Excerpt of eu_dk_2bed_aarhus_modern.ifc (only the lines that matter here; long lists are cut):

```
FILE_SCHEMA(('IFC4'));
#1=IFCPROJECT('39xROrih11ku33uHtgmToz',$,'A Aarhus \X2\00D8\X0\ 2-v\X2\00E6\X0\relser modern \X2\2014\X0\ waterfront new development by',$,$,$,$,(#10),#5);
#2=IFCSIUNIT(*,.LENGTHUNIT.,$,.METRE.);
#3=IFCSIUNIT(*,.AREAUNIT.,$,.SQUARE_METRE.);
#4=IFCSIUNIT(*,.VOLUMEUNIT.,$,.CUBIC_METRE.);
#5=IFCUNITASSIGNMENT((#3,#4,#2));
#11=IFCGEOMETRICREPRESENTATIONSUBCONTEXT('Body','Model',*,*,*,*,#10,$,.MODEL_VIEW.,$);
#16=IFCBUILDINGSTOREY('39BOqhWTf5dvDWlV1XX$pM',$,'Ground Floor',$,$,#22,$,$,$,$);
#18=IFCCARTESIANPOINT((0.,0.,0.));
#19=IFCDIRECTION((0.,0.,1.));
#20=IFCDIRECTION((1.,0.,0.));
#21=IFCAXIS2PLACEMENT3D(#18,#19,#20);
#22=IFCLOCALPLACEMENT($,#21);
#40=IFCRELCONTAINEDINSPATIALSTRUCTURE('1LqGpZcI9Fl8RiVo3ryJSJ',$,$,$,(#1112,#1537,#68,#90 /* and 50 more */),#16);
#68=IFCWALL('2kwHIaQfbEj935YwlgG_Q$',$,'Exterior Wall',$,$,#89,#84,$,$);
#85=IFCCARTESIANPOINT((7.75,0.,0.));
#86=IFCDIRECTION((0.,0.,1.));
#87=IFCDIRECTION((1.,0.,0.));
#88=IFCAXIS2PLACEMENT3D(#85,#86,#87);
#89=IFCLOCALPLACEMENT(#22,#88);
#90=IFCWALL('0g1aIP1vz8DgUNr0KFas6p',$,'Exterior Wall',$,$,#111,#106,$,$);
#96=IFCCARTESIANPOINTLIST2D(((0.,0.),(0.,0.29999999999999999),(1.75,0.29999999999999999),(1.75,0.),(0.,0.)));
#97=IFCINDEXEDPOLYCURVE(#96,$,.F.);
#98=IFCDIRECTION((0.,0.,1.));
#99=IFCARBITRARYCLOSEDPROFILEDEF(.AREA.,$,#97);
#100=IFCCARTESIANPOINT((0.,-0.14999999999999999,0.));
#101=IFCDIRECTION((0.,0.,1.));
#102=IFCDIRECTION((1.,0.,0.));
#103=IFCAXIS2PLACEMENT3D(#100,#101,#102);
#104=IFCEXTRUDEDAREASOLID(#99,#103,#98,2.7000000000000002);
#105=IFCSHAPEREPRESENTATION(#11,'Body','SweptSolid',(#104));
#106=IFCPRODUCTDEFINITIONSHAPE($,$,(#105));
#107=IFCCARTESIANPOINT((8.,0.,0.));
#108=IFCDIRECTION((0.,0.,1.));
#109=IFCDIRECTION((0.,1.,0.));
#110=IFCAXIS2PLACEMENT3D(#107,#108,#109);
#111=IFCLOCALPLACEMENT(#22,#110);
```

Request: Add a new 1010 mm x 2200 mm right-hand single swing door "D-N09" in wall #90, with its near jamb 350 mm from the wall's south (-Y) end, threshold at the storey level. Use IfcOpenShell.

```python
import numpy as np
import ifcopenshell
import ifcopenshell.api.feature
import ifcopenshell.api.geometry
import ifcopenshell.api.root
import ifcopenshell.api.spatial
import ifcopenshell.geom
import ifcopenshell.util.element
import ifcopenshell.util.placement
import ifcopenshell.util.representation
import ifcopenshell.util.shape
import ifcopenshell.util.unit

model = ifcopenshell.open("eu_dk_2bed_aarhus_modern.ifc")
unit_scale = ifcopenshell.util.unit.calculate_unit_scale(model)
settings = ifcopenshell.geom.settings()


def volume(element):
    """Net volume in cubic metres, openings subtracted."""
    shape = ifcopenshell.geom.create_shape(settings, element)
    return ifcopenshell.util.shape.get_volume(shape.geometry)


wall = model.by_guid("0g1aIP1vz8DgUNr0KFas6p")
storey = ifcopenshell.util.element.get_container(wall, ifc_class="IfcBuildingStorey")
context = ifcopenshell.util.representation.get_context(model, "Model", "Body", "MODEL_VIEW")
before = volume(wall)

width, height, from_end, sill = 1.01, 2.2, 0.35, 0.0  # metres

# The wall runs along its own X axis, and the end named is its -X end.
wall_shape = ifcopenshell.geom.create_shape(settings, wall)
x, y, z = ifcopenshell.util.shape.get_vertices(wall_shape.geometry).T
start = x.min() + from_end
face, thickness = float(y.min()), float(y.max() - y.min())
wall_matrix = ifcopenshell.util.placement.get_local_placement(wall.ObjectPlacement)
level = ifcopenshell.util.placement.get_local_placement(storey.ObjectPlacement)[2, 3]


def in_wall(x, y):
    """Placement at x, y metres in the wall's axes, at sill height."""
    matrix = wall_matrix.copy()
    matrix[:, 3] = wall_matrix @ np.array([x / unit_scale, y / unit_scale, 0.0, 1.0])
    matrix[2, 3] = level + sill / unit_scale
    return matrix


# Opening: a box that overshoots both wall faces by 50 mm.
opening = ifcopenshell.api.root.create_entity(model, ifc_class="IfcOpeningElement", predefined_type="OPENING")
box = ifcopenshell.api.geometry.add_wall_representation(
    model, context=context, length=width, height=height, thickness=thickness + 0.1
)
ifcopenshell.api.geometry.assign_representation(model, product=opening, representation=box)
ifcopenshell.api.geometry.edit_object_placement(model, product=opening, matrix=in_wall(start, face - 0.05), is_si=False)
ifcopenshell.api.feature.add_feature(model, feature=opening, element=wall)

door = ifcopenshell.api.root.create_entity(model, ifc_class="IfcDoor", name="D-N09", predefined_type="DOOR")
door.OverallWidth, door.OverallHeight = width / unit_scale, height / unit_scale
door.OperationType = "SINGLE_SWING_RIGHT"
body = ifcopenshell.api.geometry.add_door_representation(
    model,
    context=context,
    overall_width=door.OverallWidth,
    overall_height=door.OverallHeight,
    operation_type="SINGLE_SWING_RIGHT",
    lining_properties={"LiningDepth": thickness / unit_scale, "ThresholdDepth": thickness / unit_scale},
)
ifcopenshell.api.geometry.assign_representation(model, product=door, representation=body)
ifcopenshell.api.spatial.assign_container(model, products=[door], relating_structure=storey)
ifcopenshell.api.feature.add_filling(model, opening=opening, element=door)

# The lining spans the wall, so the door starts at the wall face.
ifcopenshell.api.geometry.edit_object_placement(model, product=door, matrix=in_wall(start, face), is_si=False)

after = volume(wall)

print(f"wall volume {before:.3f} -> {after:.3f} m3")

model.write("eu_dk_2bed_aarhus_modern_rev.ifc")
```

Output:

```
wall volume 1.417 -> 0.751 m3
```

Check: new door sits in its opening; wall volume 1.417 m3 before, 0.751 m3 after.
